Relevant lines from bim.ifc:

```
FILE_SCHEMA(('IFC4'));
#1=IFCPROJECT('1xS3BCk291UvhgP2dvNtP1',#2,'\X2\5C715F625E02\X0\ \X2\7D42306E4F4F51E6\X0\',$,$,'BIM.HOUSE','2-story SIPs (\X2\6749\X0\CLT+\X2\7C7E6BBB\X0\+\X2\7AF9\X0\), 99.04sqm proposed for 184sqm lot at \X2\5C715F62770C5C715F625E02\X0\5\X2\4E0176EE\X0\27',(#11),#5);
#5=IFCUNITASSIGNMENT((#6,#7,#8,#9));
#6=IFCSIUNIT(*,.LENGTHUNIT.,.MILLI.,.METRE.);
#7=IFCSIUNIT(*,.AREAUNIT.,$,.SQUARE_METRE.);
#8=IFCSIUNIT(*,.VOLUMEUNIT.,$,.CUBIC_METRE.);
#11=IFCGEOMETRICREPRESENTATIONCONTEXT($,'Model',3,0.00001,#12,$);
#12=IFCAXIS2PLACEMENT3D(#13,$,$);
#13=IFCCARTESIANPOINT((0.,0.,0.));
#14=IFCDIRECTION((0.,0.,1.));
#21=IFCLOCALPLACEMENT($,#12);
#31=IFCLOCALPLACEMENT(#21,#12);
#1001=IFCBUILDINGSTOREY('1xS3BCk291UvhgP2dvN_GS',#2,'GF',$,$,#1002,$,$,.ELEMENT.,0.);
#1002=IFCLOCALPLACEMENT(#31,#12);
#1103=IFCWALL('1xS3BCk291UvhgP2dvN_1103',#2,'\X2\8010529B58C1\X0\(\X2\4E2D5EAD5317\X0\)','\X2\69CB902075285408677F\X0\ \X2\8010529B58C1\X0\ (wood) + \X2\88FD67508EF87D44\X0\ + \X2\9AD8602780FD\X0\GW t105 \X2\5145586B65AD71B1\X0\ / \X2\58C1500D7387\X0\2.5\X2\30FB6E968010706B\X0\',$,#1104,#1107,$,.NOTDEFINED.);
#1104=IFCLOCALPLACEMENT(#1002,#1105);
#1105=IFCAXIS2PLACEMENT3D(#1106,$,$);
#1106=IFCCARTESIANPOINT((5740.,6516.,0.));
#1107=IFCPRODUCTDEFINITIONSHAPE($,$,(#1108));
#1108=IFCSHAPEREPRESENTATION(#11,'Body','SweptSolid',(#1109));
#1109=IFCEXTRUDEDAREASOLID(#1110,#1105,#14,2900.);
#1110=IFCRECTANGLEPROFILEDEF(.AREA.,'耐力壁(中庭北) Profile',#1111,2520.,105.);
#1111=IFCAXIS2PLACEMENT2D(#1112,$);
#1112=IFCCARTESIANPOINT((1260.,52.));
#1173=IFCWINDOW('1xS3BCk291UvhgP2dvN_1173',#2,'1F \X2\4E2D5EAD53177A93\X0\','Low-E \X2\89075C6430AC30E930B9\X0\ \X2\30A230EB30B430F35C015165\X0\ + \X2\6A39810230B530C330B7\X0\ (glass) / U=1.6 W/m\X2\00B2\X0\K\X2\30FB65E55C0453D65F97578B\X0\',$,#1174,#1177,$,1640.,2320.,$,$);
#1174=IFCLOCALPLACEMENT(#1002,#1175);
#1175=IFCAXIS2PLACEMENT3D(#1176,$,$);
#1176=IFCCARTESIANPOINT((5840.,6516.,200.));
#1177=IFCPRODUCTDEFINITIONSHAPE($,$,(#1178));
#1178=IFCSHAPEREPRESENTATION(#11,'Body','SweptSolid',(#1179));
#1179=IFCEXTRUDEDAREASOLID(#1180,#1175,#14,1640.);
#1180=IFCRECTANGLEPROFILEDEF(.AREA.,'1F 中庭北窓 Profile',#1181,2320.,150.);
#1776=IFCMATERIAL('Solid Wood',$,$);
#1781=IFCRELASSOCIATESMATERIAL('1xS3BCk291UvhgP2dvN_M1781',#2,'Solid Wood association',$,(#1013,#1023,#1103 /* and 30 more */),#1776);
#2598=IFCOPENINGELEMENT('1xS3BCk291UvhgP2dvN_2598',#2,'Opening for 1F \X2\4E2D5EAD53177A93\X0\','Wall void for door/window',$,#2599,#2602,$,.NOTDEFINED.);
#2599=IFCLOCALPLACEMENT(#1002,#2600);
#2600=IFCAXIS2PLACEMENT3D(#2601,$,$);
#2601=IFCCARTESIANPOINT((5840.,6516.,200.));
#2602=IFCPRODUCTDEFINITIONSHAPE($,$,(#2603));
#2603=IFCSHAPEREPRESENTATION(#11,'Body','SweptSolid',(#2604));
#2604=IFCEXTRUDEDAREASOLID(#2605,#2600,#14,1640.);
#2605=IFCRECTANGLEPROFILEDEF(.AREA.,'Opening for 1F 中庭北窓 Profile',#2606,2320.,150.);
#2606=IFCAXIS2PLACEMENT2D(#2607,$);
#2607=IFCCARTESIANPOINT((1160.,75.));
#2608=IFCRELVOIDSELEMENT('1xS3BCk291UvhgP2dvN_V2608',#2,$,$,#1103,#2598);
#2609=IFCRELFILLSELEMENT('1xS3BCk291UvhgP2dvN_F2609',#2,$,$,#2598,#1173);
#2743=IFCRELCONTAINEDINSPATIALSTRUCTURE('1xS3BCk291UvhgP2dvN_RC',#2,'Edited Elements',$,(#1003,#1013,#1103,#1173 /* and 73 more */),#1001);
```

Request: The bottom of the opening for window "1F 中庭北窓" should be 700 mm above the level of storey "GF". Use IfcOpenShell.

```python
import numpy as np
import ifcopenshell
import ifcopenshell.api.geometry
import ifcopenshell.geom
import ifcopenshell.util.element
import ifcopenshell.util.placement
import ifcopenshell.util.shape
import ifcopenshell.util.unit

model = ifcopenshell.open("bim.ifc")
unit_scale = ifcopenshell.util.unit.calculate_unit_scale(model)

window = model.by_guid("1xS3BCk291UvhgP2dvN_1173")
opening = window.FillsVoids[0].RelatingOpeningElement
storey = ifcopenshell.util.element.get_container(window, ifc_class="IfcBuildingStorey")
level = ifcopenshell.util.placement.get_local_placement(storey.ObjectPlacement)[2, 3]

# The opening's origin need not be at the sill, so measure its lowest point.
shape = ifcopenshell.geom.create_shape(ifcopenshell.geom.settings(), opening)
bottom = ifcopenshell.util.shape.get_shape_bottom_elevation(shape, shape.geometry) / unit_scale
dz = level + 0.7 / unit_scale - bottom

shift = np.array([0.0, 0.0, dz])
# The window is not placed relative to its opening, so move both.
for product in (opening, window):
    matrix = ifcopenshell.util.placement.get_local_placement(product.ObjectPlacement)
    matrix[:3, 3] += shift
    ifcopenshell.api.geometry.edit_object_placement(model, product=product, matrix=matrix, is_si=False)

print(f"moved by {dz * unit_scale:+.3f} m")

model.write("bim_edited.ifc")
```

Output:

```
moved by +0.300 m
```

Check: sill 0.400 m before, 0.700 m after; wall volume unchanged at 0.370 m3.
